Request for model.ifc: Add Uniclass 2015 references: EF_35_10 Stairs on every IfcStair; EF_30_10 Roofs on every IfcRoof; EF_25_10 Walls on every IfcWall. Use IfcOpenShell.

First a look at what the model holds.

```python
import ifcopenshell

model = ifcopenshell.open("model.ifc")
print(model.schema)
print("classifications:", [c.Name for c in model.by_type("IfcClassification")])
for ifc_class in ("IfcDoor", "IfcRoof", "IfcStair", "IfcWall", "IfcWindow"):
    print(ifc_class, len(model.by_type(ifc_class)))
```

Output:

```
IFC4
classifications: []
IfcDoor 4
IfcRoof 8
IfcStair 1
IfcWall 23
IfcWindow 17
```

```python
import ifcopenshell
import ifcopenshell.api.classification

model = ifcopenshell.open("model.ifc")

system = ifcopenshell.api.classification.add_classification(model, classification="Uniclass 2015")

codes = {
    "IfcStair": ("EF_35_10", "Stairs"),
    "IfcRoof": ("EF_30_10", "Roofs"),
    "IfcWall": ("EF_25_10", "Walls"),
}
for ifc_class, (code, name) in codes.items():
    products = model.by_type(ifc_class)
    ifcopenshell.api.classification.add_reference(
        model, products=products, classification=system, identification=code, name=name
    )
    print(code, len(products))

model.write("model_updated.ifc")
```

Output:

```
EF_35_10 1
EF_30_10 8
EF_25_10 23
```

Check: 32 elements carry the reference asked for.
